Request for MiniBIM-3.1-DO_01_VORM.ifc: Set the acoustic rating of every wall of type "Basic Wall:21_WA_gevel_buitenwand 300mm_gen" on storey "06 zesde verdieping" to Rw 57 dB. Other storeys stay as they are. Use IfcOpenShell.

First a look at what the model holds.

```python
import ifcopenshell
import ifcopenshell.util.element

model = ifcopenshell.open("MiniBIM-3.1-DO_01_VORM.ifc")
print(model.schema)
storey = next(s for s in model.by_type("IfcBuildingStorey") if s.Name == "06 zesde verdieping")
walls = [e for e in ifcopenshell.util.element.get_decomposition(storey) if e.is_a("IfcWall")]
seen = {}
for e in walls:
    element_type = ifcopenshell.util.element.get_type(e)
    key = (element_type.Name if element_type != e and element_type else None, ifcopenshell.util.element.get_pset(e, "Pset_WallCommon", "AcousticRating"))
    seen[key] = seen.get(key, 0) + 1
for (name, value), count in sorted(seen.items(), key=str):
    print(count, "x", name, "|", value)
```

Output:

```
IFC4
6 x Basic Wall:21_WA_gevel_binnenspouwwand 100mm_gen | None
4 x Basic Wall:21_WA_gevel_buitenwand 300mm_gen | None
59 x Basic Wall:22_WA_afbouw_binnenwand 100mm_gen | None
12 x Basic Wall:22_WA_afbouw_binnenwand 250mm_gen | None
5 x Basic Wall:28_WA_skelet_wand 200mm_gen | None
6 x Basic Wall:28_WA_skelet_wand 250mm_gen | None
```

```python
import ifcopenshell
import ifcopenshell.api.pset
import ifcopenshell.util.element

model = ifcopenshell.open("MiniBIM-3.1-DO_01_VORM.ifc")

storey = next(s for s in model.by_type("IfcBuildingStorey") if s.Name == "06 zesde verdieping")
walls = [e for e in ifcopenshell.util.element.get_decomposition(storey) if e.is_a("IfcWall")]

count = 0
for e in walls:
    element_type = ifcopenshell.util.element.get_type(e)
    if element_type in (None, e) or element_type.Name != "Basic Wall:21_WA_gevel_buitenwand 300mm_gen":
        continue
    # add_pset returns the element's existing set when there is one.
    pset = ifcopenshell.api.pset.add_pset(model, product=e, name="Pset_WallCommon")
    ifcopenshell.api.pset.edit_pset(model, pset=pset, properties={"AcousticRating": "Rw 57 dB"})
    count += 1

print(count, "walls updated")

model.write("MiniBIM-3.1-DO_01_VORM_v2.ifc")
```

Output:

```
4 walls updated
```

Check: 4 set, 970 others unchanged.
